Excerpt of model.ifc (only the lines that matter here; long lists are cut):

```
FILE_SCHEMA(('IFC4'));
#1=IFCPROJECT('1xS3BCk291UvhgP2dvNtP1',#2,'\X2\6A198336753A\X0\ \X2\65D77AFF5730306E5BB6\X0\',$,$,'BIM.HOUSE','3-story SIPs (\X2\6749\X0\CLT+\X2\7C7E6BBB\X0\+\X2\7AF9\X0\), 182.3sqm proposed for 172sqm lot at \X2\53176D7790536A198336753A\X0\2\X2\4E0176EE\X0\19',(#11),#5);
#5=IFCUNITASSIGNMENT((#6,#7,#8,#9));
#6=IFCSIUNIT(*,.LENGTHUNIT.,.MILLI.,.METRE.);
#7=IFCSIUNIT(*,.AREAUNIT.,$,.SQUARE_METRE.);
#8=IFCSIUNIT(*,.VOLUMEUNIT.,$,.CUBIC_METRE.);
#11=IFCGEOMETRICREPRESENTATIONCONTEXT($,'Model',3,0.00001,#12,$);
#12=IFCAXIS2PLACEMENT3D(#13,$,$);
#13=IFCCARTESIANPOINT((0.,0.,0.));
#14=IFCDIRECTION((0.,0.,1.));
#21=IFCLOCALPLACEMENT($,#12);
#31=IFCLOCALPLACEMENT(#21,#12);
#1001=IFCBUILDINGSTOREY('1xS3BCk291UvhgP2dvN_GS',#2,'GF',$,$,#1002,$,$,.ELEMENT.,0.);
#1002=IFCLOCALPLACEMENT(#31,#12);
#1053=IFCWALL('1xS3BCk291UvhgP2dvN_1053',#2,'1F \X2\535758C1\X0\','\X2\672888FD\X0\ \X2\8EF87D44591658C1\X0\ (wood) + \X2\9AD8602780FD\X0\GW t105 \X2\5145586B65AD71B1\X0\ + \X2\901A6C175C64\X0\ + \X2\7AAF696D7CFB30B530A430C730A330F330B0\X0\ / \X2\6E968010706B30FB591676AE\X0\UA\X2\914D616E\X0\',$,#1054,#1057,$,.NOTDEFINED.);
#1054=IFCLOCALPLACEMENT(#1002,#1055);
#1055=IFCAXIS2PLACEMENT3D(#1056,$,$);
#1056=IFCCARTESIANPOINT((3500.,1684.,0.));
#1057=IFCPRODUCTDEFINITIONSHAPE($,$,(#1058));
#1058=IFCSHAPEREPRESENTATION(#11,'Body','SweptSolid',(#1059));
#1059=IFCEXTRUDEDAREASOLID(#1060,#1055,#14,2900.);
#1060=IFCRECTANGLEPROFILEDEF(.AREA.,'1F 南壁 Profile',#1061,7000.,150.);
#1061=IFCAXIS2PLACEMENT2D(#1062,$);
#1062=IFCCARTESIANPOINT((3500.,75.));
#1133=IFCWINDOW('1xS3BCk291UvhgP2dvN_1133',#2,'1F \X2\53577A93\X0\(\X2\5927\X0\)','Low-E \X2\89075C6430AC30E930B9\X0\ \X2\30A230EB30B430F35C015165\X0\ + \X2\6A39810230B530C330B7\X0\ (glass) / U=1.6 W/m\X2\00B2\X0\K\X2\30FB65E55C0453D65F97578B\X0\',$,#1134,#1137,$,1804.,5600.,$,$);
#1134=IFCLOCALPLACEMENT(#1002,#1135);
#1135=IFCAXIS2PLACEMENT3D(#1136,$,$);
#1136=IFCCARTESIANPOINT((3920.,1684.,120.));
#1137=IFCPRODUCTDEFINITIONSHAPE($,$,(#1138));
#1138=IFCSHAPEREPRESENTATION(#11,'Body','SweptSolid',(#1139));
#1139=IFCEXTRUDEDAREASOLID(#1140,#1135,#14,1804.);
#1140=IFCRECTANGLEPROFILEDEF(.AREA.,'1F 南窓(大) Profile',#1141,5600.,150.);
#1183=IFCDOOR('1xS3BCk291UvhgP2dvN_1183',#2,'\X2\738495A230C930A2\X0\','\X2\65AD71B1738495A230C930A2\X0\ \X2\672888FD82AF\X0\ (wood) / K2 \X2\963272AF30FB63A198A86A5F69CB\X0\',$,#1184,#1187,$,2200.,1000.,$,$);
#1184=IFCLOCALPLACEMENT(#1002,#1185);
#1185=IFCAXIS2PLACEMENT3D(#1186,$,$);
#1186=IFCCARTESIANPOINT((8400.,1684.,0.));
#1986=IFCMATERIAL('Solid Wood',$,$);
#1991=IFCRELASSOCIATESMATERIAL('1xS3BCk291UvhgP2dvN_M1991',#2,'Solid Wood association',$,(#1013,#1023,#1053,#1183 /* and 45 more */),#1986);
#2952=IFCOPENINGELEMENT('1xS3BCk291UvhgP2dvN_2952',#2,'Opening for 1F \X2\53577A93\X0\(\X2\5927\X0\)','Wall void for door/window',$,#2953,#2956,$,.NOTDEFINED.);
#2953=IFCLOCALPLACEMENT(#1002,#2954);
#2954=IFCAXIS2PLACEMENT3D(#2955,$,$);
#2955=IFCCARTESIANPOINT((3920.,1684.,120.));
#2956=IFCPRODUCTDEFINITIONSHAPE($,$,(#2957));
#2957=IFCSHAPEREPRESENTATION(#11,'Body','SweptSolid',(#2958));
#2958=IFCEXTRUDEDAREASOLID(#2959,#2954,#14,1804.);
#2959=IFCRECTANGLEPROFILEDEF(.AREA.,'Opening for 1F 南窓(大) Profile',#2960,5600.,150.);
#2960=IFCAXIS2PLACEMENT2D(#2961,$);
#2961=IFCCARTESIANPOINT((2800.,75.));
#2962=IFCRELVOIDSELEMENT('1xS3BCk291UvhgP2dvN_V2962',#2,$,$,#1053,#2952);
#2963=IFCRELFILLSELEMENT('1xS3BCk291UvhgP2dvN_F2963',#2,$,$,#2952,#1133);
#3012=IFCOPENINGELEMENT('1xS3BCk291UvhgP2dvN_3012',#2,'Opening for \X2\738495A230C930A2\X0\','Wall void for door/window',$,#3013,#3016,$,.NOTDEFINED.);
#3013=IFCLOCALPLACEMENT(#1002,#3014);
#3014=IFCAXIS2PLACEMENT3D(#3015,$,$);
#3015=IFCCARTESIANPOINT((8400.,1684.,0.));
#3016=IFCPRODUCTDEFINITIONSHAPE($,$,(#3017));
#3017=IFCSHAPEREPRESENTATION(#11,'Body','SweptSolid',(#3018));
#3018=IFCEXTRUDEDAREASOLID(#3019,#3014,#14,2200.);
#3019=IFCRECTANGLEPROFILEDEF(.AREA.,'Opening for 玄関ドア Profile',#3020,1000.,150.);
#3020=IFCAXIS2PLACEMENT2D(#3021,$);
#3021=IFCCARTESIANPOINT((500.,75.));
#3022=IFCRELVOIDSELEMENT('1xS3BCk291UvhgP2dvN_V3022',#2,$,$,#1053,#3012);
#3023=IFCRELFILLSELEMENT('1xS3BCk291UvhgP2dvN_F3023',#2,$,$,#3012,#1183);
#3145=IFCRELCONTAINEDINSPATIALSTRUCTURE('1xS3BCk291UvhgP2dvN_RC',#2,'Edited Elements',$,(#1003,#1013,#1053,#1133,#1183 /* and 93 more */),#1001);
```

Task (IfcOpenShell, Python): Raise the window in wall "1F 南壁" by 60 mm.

```python
import numpy as np
import ifcopenshell
import ifcopenshell.api.geometry
import ifcopenshell.util.placement
import ifcopenshell.util.unit

model = ifcopenshell.open("model.ifc")
unit_scale = ifcopenshell.util.unit.calculate_unit_scale(model)

window = model.by_id(1133)
opening = window.FillsVoids[0].RelatingOpeningElement
dz = 0.06 / unit_scale

shift = np.array([0.0, 0.0, dz])
# The window is not placed relative to its opening, so move both.
for product in (opening, window):
    matrix = ifcopenshell.util.placement.get_local_placement(product.ObjectPlacement)
    matrix[:3, 3] += shift
    ifcopenshell.api.geometry.edit_object_placement(model, product=product, matrix=matrix, is_si=False)

print(f"moved by {dz * unit_scale:+.3f} m")

model.write("model_rev.ifc")
```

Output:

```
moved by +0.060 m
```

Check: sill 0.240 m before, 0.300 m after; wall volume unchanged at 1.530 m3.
